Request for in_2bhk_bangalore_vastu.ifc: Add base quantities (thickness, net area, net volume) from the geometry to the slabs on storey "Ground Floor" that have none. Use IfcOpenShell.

First a look at what the model holds.

```python
import ifcopenshell
import ifcopenshell.util.element
import ifcopenshell.util.unit

model = ifcopenshell.open("in_2bhk_bangalore_vastu.ifc")
print(model.schema)
for unit_type in ("LENGTHUNIT", "AREAUNIT", "VOLUMEUNIT"):
    print(unit_type, ifcopenshell.util.unit.calculate_unit_scale(model, unit_type))
storey = next(s for s in model.by_type("IfcBuildingStorey") if s.Name == "Ground Floor")
slabs = [e for e in ifcopenshell.util.element.get_decomposition(storey) if e.is_a("IfcSlab")]
for e in sorted(slabs, key=lambda e: e.id()):
    print(e.id(), e.is_a(), e.Name, list(ifcopenshell.util.element.get_psets(e, qtos_only=True)), sep=" | ")
```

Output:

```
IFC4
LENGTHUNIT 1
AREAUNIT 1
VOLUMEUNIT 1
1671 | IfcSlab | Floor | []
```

```python
import ifcopenshell
import ifcopenshell.api.pset
import ifcopenshell.geom
import ifcopenshell.util.element
import ifcopenshell.util.shape
import ifcopenshell.util.unit

model = ifcopenshell.open("in_2bhk_bangalore_vastu.ifc")
unit_scale = ifcopenshell.util.unit.calculate_unit_scale(model)
area_scale = ifcopenshell.util.unit.calculate_unit_scale(model, "AREAUNIT")
volume_scale = ifcopenshell.util.unit.calculate_unit_scale(model, "VOLUMEUNIT")
settings = ifcopenshell.geom.settings()

storey = next(s for s in model.by_type("IfcBuildingStorey") if s.Name == "Ground Floor")
slabs = [e for e in ifcopenshell.util.element.get_decomposition(storey) if e.is_a("IfcSlab")]

for e in sorted(slabs, key=lambda e: e.id()):
    if ifcopenshell.util.element.get_psets(e, qtos_only=True, should_inherit=False):
        continue
    # Geometry comes back in metres, in the element's own axes.
    shape = ifcopenshell.geom.create_shape(settings, e)
    values = {
        "Width": ifcopenshell.util.shape.get_z(shape.geometry) / unit_scale,
        "NetArea": ifcopenshell.util.shape.get_footprint_area(shape.geometry) / area_scale,
        "NetVolume": ifcopenshell.util.shape.get_volume(shape.geometry) / volume_scale,
    }
    qto = ifcopenshell.api.pset.add_qto(model, product=e, name="Qto_SlabBaseQuantities")
    ifcopenshell.api.pset.edit_qto(model, qto=qto, properties=values)
    print(e.id(), {k: round(v, 3) for k, v in values.items()})

model.write("in_2bhk_bangalore_vastu_edited.ifc")
```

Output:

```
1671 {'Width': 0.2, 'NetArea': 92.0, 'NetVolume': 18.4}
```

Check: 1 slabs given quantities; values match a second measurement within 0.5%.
